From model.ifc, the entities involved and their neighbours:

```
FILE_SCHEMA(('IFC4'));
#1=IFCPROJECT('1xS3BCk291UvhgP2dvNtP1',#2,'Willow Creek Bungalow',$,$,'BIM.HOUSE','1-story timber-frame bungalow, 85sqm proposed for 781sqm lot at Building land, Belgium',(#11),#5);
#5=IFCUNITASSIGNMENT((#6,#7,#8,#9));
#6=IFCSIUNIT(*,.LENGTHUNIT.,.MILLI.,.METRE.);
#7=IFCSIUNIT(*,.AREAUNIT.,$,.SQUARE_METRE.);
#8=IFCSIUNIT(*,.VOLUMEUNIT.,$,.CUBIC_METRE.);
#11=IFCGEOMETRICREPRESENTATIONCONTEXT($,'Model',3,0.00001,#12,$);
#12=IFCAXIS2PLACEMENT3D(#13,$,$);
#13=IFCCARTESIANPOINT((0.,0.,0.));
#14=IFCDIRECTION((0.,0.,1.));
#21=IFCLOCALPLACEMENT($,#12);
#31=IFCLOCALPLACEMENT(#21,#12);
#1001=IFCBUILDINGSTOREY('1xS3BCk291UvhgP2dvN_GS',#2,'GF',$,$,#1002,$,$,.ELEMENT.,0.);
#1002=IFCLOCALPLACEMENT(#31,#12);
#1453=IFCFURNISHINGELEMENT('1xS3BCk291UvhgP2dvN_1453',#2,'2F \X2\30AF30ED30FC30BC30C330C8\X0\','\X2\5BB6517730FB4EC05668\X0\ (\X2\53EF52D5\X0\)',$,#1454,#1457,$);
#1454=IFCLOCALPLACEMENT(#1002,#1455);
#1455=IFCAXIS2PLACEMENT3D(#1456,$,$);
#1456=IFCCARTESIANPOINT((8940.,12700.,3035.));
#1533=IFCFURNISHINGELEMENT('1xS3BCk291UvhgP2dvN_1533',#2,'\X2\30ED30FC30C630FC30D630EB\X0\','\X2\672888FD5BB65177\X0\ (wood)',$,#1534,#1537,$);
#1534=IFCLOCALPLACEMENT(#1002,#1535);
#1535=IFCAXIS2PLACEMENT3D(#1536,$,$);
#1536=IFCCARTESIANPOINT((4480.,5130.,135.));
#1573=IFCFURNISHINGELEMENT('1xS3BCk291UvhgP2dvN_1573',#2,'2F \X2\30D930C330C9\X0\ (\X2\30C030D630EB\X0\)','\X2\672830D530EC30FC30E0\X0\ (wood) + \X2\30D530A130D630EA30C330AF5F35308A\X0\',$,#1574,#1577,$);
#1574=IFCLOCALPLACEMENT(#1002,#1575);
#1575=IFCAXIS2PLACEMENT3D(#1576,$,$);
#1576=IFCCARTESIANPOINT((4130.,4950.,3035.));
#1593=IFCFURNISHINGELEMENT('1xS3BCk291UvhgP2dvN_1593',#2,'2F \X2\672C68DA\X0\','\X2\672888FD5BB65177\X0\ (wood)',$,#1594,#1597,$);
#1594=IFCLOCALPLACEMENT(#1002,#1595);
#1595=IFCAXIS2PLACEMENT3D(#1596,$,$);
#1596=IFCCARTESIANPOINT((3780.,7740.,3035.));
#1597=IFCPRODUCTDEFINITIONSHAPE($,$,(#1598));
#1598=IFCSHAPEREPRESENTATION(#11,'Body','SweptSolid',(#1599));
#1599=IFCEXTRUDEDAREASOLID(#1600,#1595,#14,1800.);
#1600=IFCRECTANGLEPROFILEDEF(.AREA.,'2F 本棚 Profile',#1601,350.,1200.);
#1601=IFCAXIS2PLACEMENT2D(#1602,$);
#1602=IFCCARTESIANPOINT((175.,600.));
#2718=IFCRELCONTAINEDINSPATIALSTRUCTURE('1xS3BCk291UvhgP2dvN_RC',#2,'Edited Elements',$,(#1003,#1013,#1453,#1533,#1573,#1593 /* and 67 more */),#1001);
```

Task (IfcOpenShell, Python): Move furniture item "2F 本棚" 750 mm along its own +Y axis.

```python
import ifcopenshell
import ifcopenshell.api.geometry
import ifcopenshell.util.placement

model = ifcopenshell.open("model.ifc")

item = model.by_guid("1xS3BCk291UvhgP2dvN_1593")
matrix = ifcopenshell.util.placement.get_local_placement(item.ObjectPlacement)
matrix[:3, 3] += matrix[:3, 1] * 750.0
ifcopenshell.api.geometry.edit_object_placement(model, product=item, matrix=matrix, is_si=False)

print(ifcopenshell.util.placement.get_local_placement(item.ObjectPlacement).round(3) + 0.0)

model.write("model_edited.ifc")
```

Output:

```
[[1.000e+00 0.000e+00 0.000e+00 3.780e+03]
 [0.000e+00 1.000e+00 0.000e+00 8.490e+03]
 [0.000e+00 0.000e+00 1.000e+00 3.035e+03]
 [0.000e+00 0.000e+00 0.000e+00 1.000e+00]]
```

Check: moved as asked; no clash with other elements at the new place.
